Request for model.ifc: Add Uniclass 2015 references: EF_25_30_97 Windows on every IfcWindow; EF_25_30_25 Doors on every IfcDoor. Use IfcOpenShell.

First a look at what the model holds.

```python
import ifcopenshell

model = ifcopenshell.open("model.ifc")
print(model.schema)
print("classifications:", [c.Name for c in model.by_type("IfcClassification")])
for ifc_class in ("IfcDoor", "IfcRoof", "IfcStair", "IfcWall", "IfcWindow"):
    print(ifc_class, len(model.by_type(ifc_class)))
```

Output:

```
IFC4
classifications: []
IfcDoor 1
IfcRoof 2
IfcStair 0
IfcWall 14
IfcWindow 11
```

```python
import ifcopenshell
import ifcopenshell.api.classification

model = ifcopenshell.open("model.ifc")

system = ifcopenshell.api.classification.add_classification(model, classification="Uniclass 2015")

codes = {
    "IfcWindow": ("EF_25_30_97", "Windows"),
    "IfcDoor": ("EF_25_30_25", "Doors"),
}
for ifc_class, (code, name) in codes.items():
    products = model.by_type(ifc_class)
    ifcopenshell.api.classification.add_reference(
        model, products=products, classification=system, identification=code, name=name
    )
    print(code, len(products))

model.write("model-out.ifc")
```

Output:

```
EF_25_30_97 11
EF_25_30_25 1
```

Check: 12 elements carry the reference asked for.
